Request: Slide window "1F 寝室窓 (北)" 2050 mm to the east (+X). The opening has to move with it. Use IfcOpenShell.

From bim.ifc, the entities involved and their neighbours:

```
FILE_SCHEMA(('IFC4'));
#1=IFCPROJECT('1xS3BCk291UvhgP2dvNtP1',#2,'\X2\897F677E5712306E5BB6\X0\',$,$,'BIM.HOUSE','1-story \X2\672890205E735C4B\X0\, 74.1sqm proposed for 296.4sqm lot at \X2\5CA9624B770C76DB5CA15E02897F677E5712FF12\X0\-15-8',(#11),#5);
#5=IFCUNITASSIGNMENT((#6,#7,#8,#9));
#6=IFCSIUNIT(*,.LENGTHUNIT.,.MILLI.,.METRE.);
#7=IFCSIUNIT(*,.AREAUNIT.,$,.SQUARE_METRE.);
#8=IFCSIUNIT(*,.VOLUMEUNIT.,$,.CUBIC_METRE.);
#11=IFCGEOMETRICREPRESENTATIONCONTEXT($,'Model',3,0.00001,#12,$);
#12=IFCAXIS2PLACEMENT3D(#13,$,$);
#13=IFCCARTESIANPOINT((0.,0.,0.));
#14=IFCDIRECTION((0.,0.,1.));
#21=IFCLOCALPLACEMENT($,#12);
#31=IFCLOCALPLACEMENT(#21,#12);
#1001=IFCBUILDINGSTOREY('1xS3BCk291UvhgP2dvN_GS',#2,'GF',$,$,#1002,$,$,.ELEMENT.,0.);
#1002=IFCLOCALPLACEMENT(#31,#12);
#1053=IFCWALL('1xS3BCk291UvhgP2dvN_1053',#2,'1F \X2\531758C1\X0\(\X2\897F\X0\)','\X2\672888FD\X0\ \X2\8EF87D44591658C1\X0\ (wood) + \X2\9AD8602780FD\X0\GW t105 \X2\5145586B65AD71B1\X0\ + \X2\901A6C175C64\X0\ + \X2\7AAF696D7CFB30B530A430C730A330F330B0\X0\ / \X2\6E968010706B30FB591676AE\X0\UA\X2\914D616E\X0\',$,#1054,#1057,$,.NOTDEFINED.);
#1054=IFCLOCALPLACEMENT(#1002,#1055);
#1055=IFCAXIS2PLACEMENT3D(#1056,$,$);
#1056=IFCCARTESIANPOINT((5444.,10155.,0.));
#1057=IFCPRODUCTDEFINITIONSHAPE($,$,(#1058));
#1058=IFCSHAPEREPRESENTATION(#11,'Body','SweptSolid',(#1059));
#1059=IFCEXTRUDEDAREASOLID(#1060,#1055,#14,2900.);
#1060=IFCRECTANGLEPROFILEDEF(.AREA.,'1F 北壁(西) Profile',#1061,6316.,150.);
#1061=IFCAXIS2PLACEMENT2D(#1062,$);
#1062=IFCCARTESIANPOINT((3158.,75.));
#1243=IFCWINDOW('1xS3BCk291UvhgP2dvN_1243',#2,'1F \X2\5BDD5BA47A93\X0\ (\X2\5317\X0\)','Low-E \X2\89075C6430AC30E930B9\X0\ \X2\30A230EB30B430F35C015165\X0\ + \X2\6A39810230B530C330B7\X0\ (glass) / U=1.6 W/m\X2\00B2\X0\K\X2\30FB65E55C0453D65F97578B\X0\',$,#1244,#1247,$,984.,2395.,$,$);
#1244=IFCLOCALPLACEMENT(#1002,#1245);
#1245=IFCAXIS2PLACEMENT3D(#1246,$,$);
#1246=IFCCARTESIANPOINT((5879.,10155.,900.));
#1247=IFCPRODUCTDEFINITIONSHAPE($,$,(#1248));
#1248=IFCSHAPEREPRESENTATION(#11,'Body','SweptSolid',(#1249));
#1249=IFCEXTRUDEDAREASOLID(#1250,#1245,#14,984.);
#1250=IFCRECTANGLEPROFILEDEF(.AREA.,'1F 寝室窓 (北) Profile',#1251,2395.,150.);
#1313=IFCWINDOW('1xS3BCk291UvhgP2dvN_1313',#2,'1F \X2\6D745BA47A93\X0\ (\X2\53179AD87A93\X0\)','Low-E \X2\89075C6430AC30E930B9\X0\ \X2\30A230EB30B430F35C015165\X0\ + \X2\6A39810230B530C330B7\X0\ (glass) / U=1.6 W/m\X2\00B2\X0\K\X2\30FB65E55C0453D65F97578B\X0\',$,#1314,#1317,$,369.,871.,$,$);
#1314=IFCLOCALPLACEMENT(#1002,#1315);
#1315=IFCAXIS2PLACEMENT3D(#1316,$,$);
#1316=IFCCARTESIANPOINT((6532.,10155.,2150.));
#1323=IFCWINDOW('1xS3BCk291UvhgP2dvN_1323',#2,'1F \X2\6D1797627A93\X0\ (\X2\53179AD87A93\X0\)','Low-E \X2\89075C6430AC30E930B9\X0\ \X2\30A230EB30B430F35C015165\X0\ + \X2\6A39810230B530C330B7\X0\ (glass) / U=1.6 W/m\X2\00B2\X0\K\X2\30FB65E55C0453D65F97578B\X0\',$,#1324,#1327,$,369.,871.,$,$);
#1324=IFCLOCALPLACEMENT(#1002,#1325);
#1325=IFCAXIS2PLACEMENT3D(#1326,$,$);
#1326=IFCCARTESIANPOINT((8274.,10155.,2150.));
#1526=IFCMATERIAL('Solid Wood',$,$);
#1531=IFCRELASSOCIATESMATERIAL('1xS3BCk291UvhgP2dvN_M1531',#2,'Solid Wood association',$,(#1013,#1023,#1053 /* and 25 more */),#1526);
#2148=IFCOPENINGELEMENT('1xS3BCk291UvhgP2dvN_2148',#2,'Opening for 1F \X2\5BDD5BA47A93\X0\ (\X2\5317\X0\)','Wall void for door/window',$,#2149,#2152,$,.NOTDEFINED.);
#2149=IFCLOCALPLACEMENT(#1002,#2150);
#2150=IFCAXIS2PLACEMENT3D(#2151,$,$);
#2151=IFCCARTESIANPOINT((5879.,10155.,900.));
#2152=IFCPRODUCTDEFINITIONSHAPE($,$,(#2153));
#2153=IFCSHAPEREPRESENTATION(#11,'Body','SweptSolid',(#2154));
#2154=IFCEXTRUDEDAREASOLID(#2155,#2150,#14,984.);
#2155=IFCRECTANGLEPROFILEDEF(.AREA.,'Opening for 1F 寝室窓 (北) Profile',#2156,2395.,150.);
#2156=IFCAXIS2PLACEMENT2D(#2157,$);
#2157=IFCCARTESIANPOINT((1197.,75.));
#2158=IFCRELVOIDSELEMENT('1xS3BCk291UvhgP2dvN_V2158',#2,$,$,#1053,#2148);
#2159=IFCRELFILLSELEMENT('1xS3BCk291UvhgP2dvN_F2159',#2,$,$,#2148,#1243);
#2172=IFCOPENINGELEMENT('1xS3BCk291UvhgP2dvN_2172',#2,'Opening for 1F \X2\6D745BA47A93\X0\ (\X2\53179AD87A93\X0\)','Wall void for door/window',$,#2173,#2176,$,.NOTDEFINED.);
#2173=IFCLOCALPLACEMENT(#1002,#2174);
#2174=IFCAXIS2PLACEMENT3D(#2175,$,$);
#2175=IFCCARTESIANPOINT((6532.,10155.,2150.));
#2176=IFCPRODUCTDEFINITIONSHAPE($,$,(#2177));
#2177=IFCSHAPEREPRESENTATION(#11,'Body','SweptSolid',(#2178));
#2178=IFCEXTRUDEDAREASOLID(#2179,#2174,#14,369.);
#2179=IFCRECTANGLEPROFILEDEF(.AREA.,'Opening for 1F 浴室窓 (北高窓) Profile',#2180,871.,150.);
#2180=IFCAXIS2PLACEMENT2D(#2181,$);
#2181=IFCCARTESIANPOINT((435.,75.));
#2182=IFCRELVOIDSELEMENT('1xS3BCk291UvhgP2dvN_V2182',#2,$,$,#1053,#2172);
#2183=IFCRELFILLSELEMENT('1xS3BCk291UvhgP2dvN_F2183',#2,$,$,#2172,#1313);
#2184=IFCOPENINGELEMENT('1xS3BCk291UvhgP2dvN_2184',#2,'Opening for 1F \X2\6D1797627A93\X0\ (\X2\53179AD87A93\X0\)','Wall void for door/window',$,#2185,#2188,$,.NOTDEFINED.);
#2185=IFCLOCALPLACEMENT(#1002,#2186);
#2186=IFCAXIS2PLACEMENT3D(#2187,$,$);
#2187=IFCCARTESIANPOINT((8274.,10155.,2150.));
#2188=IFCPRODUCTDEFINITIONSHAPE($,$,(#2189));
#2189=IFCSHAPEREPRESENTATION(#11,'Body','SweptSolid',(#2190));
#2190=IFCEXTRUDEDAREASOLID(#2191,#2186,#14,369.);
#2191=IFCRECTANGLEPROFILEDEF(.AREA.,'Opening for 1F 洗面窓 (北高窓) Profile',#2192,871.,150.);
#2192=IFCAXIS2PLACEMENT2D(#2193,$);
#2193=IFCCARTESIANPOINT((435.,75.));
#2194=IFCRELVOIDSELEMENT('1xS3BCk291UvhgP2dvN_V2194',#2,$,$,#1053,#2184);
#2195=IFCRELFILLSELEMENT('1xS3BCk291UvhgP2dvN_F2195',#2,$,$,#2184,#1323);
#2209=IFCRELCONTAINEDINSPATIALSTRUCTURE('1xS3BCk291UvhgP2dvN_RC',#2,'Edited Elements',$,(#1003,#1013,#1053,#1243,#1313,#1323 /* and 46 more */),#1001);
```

```python
import ifcopenshell
import ifcopenshell.api.geometry
import ifcopenshell.util.placement

model = ifcopenshell.open("bim.ifc")

window = model.by_guid("1xS3BCk291UvhgP2dvN_1243")
opening = window.FillsVoids[0].RelatingOpeningElement
wall = opening.VoidsElements[0].RelatingBuildingElement

wall_matrix = ifcopenshell.util.placement.get_local_placement(wall.ObjectPlacement)
shift = wall_matrix[:3, 0] * 2050.0
before = ifcopenshell.util.placement.get_local_placement(window.ObjectPlacement)[:3, 3].copy()

# The window is not placed relative to its opening, so move both.
for product in (opening, window):
    matrix = ifcopenshell.util.placement.get_local_placement(product.ObjectPlacement)
    matrix[:3, 3] += shift
    ifcopenshell.api.geometry.edit_object_placement(model, product=product, matrix=matrix, is_si=False)

after = ifcopenshell.util.placement.get_local_placement(window.ObjectPlacement)[:3, 3]
print("window moved by", (after - before).round(3) + 0.0)

model.write("bim_updated.ifc")
```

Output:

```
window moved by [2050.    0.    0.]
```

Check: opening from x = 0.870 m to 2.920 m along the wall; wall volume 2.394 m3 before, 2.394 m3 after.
